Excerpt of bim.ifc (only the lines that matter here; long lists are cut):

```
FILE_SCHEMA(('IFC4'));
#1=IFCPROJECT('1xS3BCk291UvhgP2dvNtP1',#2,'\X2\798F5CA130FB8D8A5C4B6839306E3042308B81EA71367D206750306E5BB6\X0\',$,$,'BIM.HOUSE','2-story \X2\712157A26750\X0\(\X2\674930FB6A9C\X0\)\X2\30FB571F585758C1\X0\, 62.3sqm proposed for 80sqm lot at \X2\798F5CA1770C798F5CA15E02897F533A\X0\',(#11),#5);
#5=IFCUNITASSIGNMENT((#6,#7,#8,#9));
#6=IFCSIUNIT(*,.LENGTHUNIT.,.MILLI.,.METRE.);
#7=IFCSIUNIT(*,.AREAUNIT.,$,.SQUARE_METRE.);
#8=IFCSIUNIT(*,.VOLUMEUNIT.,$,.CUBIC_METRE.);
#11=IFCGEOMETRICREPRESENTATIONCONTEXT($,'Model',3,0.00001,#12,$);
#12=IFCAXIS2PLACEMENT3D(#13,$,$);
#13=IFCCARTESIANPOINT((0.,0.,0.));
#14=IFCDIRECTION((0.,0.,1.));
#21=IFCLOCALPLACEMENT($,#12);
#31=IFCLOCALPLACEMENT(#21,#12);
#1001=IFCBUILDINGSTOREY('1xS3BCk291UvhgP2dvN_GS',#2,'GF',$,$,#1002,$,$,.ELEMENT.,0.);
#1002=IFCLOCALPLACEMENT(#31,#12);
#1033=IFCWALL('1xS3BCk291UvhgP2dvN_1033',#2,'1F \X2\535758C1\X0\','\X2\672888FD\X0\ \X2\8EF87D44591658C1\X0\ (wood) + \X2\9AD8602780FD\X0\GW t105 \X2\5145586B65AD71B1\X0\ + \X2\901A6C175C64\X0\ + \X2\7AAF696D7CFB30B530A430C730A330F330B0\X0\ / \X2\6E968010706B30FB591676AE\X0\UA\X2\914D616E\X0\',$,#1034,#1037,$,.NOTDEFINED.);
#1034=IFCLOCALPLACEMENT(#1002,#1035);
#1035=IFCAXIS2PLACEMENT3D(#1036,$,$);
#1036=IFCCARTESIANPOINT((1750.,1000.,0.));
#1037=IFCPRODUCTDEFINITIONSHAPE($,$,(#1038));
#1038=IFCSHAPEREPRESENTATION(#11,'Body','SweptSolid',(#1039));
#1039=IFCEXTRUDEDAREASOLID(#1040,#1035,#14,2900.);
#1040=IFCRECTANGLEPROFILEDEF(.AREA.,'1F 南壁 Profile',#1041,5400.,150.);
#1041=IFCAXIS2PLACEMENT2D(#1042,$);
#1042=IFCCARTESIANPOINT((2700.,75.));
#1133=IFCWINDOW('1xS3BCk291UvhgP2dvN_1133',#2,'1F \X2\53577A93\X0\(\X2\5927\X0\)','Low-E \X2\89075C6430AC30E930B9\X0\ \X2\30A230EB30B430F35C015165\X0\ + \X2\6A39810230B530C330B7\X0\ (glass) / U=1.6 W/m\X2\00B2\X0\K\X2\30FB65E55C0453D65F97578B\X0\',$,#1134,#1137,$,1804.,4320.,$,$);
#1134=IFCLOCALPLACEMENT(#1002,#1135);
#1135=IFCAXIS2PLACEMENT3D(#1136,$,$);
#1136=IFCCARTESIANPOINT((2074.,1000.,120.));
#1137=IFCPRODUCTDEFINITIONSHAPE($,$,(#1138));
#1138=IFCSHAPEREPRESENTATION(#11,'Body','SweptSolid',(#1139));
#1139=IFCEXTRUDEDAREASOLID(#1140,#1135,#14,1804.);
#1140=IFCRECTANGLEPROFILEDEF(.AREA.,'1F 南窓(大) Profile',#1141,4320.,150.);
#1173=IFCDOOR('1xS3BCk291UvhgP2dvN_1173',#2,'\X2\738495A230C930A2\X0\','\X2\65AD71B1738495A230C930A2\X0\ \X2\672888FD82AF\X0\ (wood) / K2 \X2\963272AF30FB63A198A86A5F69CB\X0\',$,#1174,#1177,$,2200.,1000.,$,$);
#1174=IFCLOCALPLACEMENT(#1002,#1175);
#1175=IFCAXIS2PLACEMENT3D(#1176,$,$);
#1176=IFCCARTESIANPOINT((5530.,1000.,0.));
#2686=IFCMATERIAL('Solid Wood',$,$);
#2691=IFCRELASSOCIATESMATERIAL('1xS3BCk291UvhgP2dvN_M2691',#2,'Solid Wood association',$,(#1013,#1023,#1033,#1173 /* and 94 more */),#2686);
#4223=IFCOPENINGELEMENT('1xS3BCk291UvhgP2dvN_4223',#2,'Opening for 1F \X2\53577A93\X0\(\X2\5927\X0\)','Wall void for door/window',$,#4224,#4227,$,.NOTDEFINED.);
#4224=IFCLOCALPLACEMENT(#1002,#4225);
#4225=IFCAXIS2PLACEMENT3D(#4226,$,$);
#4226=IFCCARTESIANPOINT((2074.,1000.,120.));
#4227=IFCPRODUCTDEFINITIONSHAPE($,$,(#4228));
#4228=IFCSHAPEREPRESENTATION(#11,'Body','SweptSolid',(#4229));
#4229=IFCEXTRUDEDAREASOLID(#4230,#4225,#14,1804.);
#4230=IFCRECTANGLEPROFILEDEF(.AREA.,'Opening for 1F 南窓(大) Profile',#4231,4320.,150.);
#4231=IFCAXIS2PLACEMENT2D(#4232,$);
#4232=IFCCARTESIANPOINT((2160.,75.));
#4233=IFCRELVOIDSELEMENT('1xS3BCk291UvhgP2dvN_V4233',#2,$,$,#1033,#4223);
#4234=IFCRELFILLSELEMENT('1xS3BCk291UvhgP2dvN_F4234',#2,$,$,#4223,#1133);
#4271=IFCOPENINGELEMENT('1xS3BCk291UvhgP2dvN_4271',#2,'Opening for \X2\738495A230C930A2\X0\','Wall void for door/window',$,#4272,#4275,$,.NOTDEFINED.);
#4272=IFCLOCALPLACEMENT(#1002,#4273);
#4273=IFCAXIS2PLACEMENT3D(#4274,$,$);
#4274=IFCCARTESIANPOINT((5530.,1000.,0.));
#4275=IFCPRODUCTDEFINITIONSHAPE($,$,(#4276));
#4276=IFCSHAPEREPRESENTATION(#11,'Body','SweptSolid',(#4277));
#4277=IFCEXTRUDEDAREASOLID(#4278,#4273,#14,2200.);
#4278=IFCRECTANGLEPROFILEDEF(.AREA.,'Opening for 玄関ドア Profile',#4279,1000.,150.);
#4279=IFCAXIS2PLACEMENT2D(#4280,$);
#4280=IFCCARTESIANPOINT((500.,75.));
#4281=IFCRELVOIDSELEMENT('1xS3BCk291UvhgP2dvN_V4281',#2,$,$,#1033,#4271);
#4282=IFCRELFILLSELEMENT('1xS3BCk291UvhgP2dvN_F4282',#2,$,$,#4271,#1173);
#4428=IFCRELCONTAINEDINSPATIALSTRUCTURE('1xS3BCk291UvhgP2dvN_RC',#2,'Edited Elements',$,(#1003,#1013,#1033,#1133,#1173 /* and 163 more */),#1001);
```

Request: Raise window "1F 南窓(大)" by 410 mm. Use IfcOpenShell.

```python
import numpy as np
import ifcopenshell
import ifcopenshell.api.geometry
import ifcopenshell.util.placement
import ifcopenshell.util.unit

model = ifcopenshell.open("bim.ifc")
unit_scale = ifcopenshell.util.unit.calculate_unit_scale(model)

window = model.by_guid("1xS3BCk291UvhgP2dvN_1133")
opening = window.FillsVoids[0].RelatingOpeningElement
dz = 0.41 / unit_scale

shift = np.array([0.0, 0.0, dz])
# The window is not placed relative to its opening, so move both.
for product in (opening, window):
    matrix = ifcopenshell.util.placement.get_local_placement(product.ObjectPlacement)
    matrix[:3, 3] += shift
    ifcopenshell.api.geometry.edit_object_placement(model, product=product, matrix=matrix, is_si=False)

print(f"moved by {dz * unit_scale:+.3f} m")

model.write("bim_edited.ifc")
```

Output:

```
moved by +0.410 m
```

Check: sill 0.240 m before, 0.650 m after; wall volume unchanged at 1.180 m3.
